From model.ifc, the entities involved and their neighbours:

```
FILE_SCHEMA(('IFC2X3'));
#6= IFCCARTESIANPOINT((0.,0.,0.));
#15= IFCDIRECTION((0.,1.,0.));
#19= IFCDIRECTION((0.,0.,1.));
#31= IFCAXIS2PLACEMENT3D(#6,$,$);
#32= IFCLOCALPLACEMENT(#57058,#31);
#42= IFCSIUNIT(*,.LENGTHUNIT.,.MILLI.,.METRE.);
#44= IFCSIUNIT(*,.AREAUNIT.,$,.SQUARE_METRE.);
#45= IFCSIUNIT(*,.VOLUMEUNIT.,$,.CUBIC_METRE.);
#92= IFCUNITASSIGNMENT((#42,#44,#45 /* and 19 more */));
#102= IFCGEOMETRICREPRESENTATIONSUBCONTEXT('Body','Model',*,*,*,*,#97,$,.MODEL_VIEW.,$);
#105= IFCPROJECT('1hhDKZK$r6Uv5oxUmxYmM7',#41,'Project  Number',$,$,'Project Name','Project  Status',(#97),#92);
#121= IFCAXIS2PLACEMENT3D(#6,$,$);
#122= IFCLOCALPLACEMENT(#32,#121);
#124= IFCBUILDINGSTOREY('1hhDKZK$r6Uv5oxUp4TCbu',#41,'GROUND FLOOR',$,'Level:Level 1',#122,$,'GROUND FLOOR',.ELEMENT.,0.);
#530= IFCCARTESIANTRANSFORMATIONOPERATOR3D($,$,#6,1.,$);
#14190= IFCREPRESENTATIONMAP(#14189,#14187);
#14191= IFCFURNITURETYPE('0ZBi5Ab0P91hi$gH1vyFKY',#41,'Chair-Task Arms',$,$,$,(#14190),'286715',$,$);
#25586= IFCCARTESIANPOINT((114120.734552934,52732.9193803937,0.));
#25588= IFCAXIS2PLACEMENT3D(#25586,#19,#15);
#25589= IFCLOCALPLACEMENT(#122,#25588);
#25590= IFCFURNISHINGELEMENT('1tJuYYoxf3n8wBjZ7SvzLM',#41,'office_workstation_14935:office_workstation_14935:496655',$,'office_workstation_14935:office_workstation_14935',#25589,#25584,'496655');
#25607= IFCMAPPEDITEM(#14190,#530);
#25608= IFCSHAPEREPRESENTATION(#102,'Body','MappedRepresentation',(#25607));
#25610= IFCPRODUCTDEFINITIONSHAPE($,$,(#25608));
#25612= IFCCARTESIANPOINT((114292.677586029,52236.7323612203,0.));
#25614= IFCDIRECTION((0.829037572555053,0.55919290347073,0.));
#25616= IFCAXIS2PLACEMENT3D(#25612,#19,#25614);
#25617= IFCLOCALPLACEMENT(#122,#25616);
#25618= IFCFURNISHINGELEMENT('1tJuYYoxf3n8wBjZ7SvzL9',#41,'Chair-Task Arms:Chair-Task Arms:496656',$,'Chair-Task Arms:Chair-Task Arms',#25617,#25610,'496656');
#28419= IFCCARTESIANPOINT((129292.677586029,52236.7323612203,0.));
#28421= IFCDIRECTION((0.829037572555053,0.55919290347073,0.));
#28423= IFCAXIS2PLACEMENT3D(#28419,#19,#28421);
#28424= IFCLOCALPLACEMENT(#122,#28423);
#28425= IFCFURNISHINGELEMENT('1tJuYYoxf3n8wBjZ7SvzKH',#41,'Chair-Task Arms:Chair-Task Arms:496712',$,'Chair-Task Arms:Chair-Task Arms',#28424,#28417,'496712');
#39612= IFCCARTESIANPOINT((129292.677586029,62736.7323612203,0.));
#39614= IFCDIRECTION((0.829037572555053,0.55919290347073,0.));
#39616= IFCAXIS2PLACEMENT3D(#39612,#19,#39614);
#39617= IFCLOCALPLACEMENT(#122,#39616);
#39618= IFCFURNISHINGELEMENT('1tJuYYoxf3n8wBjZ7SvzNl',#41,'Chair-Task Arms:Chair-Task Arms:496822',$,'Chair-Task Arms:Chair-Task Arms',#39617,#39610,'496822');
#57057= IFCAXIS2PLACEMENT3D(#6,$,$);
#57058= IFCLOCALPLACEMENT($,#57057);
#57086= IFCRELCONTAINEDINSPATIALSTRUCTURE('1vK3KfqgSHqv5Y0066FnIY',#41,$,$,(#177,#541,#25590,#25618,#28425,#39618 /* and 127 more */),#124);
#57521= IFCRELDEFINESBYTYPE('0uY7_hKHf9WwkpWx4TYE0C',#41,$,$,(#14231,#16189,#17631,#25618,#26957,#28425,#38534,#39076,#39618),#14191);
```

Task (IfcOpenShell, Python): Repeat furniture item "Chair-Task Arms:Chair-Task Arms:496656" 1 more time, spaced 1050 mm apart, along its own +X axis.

```python
import ifcopenshell
import ifcopenshell.api.geometry
import ifcopenshell.api.root
import ifcopenshell.util.element
import ifcopenshell.util.placement

model = ifcopenshell.open("model.ifc")


def reuse_history(source, copy):
    """copy_class also copies each property set's owner history, people and application; keep the originals."""
    for rel in copy.IsDefinedBy:
        if rel.is_a("IfcRelDefinesByProperties") and (history := rel.RelatingPropertyDefinition.OwnerHistory):
            rel.RelatingPropertyDefinition.OwnerHistory = source.OwnerHistory
            ifcopenshell.util.element.remove_deep2(model, history)


source = model.by_guid("1tJuYYoxf3n8wBjZ7SvzL9")
base = ifcopenshell.util.placement.get_local_placement(source.ObjectPlacement)
step = base[:3, 0] * 1050.0

for i in range(1, 2):
    copy = ifcopenshell.api.root.copy_class(model, product=source)
    copy.Representation = ifcopenshell.util.element.copy_deep(
        model, source.Representation, exclude=["IfcGeometricRepresentationContext", "IfcRepresentationMap"]
    )
    copy.Name = "Chair-Task Arms:Chair-Task Arms"
    copy.Tag = None
    reuse_history(source, copy)
    matrix = base.copy()
    matrix[:3, 3] += i * step
    print("added at", matrix[:3, 3].round(3) + 0.0)
    ifcopenshell.api.geometry.edit_object_placement(model, product=copy, matrix=matrix, is_si=False)

model.write("model_v2.ifc")
```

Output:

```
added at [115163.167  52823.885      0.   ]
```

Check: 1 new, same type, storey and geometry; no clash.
